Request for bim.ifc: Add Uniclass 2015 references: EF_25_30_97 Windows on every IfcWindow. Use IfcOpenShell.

First a look at what the model holds.

```python
import ifcopenshell

model = ifcopenshell.open("bim.ifc")
print(model.schema)
print("classifications:", [c.Name for c in model.by_type("IfcClassification")])
for ifc_class in ("IfcDoor", "IfcRoof", "IfcStair", "IfcWall", "IfcWindow"):
    print(ifc_class, len(model.by_type(ifc_class)))
```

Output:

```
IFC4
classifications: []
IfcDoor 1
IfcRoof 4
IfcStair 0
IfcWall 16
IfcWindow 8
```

```python
import ifcopenshell
import ifcopenshell.api.classification

model = ifcopenshell.open("bim.ifc")

system = ifcopenshell.api.classification.add_classification(model, classification="Uniclass 2015")

codes = {
    "IfcWindow": ("EF_25_30_97", "Windows"),
}
for ifc_class, (code, name) in codes.items():
    products = model.by_type(ifc_class)
    ifcopenshell.api.classification.add_reference(
        model, products=products, classification=system, identification=code, name=name
    )
    print(code, len(products))

model.write("bim_edited.ifc")
```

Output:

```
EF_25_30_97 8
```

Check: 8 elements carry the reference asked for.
